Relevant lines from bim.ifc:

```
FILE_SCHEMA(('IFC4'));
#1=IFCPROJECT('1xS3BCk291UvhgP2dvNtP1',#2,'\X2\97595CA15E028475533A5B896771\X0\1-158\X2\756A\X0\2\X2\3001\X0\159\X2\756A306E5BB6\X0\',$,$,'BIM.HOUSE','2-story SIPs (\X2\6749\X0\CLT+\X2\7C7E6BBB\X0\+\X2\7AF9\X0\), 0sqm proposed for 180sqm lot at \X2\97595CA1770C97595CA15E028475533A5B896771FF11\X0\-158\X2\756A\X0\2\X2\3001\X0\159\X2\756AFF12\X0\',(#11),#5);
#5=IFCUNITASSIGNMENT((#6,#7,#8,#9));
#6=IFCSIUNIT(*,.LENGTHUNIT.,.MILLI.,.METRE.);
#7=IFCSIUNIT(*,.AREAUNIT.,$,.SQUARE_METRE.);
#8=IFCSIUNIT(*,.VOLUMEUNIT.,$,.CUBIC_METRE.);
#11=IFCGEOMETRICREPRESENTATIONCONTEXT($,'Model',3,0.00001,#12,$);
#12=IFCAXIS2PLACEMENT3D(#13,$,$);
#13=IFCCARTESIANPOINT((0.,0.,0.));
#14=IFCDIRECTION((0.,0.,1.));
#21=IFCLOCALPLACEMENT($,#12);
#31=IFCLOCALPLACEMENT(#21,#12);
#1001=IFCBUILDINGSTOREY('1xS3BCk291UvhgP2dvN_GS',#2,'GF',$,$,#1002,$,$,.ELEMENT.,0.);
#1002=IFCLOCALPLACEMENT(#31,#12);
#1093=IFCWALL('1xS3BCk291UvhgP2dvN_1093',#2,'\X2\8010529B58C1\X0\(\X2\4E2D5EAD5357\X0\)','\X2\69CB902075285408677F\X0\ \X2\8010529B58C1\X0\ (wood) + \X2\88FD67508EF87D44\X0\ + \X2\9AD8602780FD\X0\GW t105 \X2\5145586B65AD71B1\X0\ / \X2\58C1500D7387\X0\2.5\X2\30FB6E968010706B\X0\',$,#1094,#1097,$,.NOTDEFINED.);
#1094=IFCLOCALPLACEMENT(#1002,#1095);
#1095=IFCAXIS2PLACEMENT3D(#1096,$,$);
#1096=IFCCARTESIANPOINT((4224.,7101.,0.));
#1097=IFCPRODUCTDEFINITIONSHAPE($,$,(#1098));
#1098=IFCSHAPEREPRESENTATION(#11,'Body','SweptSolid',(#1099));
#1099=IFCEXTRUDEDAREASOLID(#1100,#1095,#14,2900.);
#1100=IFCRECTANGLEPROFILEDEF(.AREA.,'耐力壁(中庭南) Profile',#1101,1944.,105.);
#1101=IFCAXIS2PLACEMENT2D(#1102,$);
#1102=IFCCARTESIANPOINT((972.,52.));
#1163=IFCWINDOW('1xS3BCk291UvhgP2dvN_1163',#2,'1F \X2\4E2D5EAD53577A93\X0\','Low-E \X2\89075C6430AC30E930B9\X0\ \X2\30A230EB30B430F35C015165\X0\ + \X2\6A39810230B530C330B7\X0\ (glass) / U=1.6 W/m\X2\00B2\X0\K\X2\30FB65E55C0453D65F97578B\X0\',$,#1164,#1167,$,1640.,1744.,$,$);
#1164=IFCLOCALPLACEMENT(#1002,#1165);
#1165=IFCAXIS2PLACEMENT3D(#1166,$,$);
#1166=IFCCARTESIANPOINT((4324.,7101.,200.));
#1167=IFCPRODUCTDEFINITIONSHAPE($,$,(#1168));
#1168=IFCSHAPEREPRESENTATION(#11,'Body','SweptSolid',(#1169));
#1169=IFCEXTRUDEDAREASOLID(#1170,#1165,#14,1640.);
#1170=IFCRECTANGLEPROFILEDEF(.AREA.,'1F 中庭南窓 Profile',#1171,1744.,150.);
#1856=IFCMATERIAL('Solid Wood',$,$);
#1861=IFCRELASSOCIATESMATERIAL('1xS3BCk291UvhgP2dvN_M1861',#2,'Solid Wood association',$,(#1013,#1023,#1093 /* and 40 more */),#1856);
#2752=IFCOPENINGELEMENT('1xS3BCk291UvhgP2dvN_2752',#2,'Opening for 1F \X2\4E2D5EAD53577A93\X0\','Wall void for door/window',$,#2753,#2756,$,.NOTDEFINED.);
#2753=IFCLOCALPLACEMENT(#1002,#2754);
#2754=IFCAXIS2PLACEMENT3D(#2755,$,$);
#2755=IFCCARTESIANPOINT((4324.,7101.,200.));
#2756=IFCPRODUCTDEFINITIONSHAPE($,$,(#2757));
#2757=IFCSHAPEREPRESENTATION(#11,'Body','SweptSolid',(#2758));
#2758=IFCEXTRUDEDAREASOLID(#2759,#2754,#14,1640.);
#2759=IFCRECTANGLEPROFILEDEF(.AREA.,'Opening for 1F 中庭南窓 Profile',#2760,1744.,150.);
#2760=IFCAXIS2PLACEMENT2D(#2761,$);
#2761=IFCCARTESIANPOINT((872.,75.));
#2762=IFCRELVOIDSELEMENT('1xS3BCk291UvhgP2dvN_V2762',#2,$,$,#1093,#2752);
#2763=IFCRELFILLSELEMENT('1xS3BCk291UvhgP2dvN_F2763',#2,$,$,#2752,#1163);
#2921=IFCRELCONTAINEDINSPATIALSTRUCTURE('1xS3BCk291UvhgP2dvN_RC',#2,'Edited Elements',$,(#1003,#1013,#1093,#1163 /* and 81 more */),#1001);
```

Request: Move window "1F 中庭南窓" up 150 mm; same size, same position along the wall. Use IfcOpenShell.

```python
import numpy as np
import ifcopenshell
import ifcopenshell.api.geometry
import ifcopenshell.util.placement
import ifcopenshell.util.unit

model = ifcopenshell.open("bim.ifc")
unit_scale = ifcopenshell.util.unit.calculate_unit_scale(model)

window = model.by_guid("1xS3BCk291UvhgP2dvN_1163")
opening = window.FillsVoids[0].RelatingOpeningElement
dz = 0.15 / unit_scale

shift = np.array([0.0, 0.0, dz])
# The window is not placed relative to its opening, so move both.
for product in (opening, window):
    matrix = ifcopenshell.util.placement.get_local_placement(product.ObjectPlacement)
    matrix[:3, 3] += shift
    ifcopenshell.api.geometry.edit_object_placement(model, product=product, matrix=matrix, is_si=False)

print(f"moved by {dz * unit_scale:+.3f} m")

model.write("bim_rev.ifc")
```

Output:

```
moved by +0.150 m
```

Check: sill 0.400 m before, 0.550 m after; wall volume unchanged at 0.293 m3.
